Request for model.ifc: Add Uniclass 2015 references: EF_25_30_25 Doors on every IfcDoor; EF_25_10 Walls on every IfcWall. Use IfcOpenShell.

First a look at what the model holds.

```python
import ifcopenshell

model = ifcopenshell.open("model.ifc")
print(model.schema)
print("classifications:", [c.Name for c in model.by_type("IfcClassification")])
for ifc_class in ("IfcDoor", "IfcRoof", "IfcStair", "IfcWall", "IfcWindow"):
    print(ifc_class, len(model.by_type(ifc_class)))
```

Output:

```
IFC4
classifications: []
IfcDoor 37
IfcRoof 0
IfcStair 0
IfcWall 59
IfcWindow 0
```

```python
import ifcopenshell
import ifcopenshell.api.classification

model = ifcopenshell.open("model.ifc")

system = ifcopenshell.api.classification.add_classification(model, classification="Uniclass 2015")

codes = {
    "IfcDoor": ("EF_25_30_25", "Doors"),
    "IfcWall": ("EF_25_10", "Walls"),
}
for ifc_class, (code, name) in codes.items():
    products = model.by_type(ifc_class)
    ifcopenshell.api.classification.add_reference(
        model, products=products, classification=system, identification=code, name=name
    )
    print(code, len(products))

model.write("model_updated.ifc")
```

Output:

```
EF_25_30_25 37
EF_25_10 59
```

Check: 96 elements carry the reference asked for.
